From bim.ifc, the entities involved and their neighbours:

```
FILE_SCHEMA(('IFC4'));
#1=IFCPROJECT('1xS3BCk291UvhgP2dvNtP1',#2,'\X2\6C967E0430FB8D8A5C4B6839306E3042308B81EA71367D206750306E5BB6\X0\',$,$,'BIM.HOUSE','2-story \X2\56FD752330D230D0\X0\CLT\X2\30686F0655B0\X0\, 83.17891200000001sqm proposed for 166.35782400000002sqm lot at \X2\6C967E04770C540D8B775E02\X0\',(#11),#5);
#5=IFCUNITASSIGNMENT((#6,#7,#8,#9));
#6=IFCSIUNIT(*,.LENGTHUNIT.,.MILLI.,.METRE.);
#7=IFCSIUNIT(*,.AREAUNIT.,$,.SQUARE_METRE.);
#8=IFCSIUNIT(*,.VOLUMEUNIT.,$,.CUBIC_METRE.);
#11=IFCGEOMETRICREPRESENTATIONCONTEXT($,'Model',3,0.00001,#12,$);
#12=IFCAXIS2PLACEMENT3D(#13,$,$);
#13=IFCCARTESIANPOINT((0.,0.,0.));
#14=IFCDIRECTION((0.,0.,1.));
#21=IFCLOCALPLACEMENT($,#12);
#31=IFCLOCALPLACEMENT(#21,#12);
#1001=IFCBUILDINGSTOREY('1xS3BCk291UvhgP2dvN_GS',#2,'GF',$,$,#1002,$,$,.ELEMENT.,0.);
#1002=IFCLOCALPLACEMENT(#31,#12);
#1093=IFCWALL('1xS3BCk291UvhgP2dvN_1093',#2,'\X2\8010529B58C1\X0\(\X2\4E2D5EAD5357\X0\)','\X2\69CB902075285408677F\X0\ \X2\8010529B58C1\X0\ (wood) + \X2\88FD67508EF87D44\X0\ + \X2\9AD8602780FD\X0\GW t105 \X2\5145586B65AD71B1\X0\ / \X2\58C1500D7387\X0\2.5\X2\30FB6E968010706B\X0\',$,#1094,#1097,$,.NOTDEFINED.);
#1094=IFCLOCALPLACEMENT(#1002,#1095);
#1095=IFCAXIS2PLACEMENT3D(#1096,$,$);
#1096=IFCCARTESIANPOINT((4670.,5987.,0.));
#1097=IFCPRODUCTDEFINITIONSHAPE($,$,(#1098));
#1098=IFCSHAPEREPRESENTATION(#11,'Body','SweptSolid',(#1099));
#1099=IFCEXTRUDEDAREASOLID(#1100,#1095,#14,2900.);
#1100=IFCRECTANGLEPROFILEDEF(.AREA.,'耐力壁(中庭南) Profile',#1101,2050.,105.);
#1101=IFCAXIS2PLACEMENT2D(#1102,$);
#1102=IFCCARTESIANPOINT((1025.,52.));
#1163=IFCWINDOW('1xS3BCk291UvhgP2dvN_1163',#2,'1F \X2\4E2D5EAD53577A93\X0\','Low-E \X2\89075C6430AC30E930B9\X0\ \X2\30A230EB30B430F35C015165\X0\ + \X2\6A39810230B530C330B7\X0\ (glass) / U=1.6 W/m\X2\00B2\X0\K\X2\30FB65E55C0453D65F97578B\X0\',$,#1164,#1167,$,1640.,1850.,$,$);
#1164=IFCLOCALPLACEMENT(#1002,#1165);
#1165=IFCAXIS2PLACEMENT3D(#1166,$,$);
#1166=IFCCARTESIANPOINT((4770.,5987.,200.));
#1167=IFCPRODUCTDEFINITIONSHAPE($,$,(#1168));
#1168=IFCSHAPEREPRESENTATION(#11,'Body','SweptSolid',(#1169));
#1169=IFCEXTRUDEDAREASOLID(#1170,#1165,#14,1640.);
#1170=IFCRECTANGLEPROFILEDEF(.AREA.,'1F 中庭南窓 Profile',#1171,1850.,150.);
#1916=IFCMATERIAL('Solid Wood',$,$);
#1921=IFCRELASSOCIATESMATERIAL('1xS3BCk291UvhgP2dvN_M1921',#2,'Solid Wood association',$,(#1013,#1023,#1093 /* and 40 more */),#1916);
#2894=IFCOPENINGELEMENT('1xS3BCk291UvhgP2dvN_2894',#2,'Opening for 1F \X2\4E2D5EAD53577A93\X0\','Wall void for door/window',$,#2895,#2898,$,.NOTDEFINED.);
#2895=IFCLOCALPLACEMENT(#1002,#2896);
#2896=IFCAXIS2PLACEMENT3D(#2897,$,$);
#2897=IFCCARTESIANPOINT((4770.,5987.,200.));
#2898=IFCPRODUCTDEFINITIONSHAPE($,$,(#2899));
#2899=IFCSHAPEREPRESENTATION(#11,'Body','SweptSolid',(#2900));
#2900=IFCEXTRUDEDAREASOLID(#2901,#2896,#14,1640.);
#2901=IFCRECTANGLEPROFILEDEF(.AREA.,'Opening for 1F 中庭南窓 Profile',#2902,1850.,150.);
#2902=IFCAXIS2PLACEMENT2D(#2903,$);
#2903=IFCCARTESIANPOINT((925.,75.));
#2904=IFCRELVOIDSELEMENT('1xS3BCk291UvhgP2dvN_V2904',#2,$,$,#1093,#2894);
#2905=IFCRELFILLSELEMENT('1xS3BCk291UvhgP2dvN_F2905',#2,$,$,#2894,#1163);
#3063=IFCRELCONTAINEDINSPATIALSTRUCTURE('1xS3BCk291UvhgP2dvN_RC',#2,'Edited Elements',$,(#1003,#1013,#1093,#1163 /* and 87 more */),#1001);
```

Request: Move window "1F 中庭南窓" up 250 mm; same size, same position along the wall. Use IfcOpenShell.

```python
import numpy as np
import ifcopenshell
import ifcopenshell.api.geometry
import ifcopenshell.util.placement
import ifcopenshell.util.unit

model = ifcopenshell.open("bim.ifc")
unit_scale = ifcopenshell.util.unit.calculate_unit_scale(model)

window = model.by_id(1163)
opening = window.FillsVoids[0].RelatingOpeningElement
dz = 250.0

shift = np.array([0.0, 0.0, dz])
# The window is not placed relative to its opening, so move both.
for product in (opening, window):
    matrix = ifcopenshell.util.placement.get_local_placement(product.ObjectPlacement)
    matrix[:3, 3] += shift
    ifcopenshell.api.geometry.edit_object_placement(model, product=product, matrix=matrix, is_si=False)

print(f"moved by {dz * unit_scale:+.3f} m")

model.write("bim_rev.ifc")
```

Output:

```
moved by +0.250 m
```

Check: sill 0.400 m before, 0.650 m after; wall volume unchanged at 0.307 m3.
